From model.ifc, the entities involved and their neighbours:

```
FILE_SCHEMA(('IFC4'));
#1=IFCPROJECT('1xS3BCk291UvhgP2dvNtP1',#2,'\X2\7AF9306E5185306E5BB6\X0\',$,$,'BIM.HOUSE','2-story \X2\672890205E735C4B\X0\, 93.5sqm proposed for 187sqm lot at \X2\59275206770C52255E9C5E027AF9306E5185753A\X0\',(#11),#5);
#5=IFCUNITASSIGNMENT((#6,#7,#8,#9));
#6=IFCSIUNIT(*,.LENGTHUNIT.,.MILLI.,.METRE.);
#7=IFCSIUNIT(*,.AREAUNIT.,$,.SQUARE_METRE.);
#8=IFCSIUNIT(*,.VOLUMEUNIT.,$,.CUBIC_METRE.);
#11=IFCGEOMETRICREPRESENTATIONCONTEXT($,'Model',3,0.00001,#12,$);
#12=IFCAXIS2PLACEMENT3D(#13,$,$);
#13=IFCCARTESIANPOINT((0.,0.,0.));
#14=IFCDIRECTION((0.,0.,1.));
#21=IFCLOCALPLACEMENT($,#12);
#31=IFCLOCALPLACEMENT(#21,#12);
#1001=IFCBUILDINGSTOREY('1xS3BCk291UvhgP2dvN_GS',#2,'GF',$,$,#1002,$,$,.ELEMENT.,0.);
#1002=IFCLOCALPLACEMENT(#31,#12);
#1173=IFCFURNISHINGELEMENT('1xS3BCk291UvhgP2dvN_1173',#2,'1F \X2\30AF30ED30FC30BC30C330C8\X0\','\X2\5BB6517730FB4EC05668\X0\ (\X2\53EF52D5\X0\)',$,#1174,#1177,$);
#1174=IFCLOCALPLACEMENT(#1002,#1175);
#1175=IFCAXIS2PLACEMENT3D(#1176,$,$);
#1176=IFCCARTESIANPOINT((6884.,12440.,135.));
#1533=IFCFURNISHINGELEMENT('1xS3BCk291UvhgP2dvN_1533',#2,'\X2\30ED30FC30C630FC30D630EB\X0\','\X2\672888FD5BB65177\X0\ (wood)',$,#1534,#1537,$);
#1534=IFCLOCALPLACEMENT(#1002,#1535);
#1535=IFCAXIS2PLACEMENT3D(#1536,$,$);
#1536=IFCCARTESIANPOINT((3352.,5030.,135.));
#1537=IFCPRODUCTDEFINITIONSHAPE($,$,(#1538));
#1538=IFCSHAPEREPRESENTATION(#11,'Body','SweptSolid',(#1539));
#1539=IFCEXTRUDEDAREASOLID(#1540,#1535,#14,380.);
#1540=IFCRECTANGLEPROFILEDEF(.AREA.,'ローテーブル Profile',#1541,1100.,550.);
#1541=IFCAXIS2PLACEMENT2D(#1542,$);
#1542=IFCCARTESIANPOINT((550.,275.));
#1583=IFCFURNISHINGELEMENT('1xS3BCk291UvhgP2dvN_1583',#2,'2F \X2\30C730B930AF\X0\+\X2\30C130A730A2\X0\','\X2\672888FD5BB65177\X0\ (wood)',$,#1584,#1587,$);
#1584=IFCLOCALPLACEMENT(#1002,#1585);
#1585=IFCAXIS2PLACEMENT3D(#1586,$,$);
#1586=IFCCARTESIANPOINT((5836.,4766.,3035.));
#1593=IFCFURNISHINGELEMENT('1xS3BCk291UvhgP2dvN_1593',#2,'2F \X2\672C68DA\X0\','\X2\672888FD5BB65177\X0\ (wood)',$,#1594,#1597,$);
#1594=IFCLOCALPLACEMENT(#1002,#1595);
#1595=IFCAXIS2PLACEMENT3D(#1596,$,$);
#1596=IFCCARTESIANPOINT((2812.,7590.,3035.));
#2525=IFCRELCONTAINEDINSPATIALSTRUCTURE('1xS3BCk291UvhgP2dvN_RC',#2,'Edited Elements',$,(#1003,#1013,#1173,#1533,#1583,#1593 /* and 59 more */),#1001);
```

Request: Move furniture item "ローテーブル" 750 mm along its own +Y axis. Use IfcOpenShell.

```python
import ifcopenshell
import ifcopenshell.api.geometry
import ifcopenshell.util.placement

model = ifcopenshell.open("model.ifc")

item = model.by_id(1533)
matrix = ifcopenshell.util.placement.get_local_placement(item.ObjectPlacement)
matrix[:3, 3] += matrix[:3, 1] * 750.0
ifcopenshell.api.geometry.edit_object_placement(model, product=item, matrix=matrix, is_si=False)

print(ifcopenshell.util.placement.get_local_placement(item.ObjectPlacement).round(3) + 0.0)

model.write("model_edited.ifc")
```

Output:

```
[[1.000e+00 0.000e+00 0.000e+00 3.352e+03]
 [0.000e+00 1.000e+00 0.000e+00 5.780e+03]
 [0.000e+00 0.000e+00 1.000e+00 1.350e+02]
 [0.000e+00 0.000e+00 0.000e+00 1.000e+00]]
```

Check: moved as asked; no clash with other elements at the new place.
